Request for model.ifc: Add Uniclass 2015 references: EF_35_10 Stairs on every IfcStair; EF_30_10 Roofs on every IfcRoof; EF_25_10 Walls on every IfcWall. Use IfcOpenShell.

First a look at what the model holds.

```python
import ifcopenshell

model = ifcopenshell.open("model.ifc")
print(model.schema)
print("classifications:", [c.Name for c in model.by_type("IfcClassification")])
for ifc_class in ("IfcDoor", "IfcRoof", "IfcStair", "IfcWall", "IfcWindow"):
    print(ifc_class, len(model.by_type(ifc_class)))
```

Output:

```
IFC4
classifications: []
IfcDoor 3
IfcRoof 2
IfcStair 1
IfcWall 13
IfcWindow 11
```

```python
import ifcopenshell
import ifcopenshell.api.classification

model = ifcopenshell.open("model.ifc")

system = ifcopenshell.api.classification.add_classification(model, classification="Uniclass 2015")

codes = {
    "IfcStair": ("EF_35_10", "Stairs"),
    "IfcRoof": ("EF_30_10", "Roofs"),
    "IfcWall": ("EF_25_10", "Walls"),
}
for ifc_class, (code, name) in codes.items():
    products = model.by_type(ifc_class)
    ifcopenshell.api.classification.add_reference(
        model, products=products, classification=system, identification=code, name=name
    )
    print(code, len(products))

model.write("model_rev.ifc")
```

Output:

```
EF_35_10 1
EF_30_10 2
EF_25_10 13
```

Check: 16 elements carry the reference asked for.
